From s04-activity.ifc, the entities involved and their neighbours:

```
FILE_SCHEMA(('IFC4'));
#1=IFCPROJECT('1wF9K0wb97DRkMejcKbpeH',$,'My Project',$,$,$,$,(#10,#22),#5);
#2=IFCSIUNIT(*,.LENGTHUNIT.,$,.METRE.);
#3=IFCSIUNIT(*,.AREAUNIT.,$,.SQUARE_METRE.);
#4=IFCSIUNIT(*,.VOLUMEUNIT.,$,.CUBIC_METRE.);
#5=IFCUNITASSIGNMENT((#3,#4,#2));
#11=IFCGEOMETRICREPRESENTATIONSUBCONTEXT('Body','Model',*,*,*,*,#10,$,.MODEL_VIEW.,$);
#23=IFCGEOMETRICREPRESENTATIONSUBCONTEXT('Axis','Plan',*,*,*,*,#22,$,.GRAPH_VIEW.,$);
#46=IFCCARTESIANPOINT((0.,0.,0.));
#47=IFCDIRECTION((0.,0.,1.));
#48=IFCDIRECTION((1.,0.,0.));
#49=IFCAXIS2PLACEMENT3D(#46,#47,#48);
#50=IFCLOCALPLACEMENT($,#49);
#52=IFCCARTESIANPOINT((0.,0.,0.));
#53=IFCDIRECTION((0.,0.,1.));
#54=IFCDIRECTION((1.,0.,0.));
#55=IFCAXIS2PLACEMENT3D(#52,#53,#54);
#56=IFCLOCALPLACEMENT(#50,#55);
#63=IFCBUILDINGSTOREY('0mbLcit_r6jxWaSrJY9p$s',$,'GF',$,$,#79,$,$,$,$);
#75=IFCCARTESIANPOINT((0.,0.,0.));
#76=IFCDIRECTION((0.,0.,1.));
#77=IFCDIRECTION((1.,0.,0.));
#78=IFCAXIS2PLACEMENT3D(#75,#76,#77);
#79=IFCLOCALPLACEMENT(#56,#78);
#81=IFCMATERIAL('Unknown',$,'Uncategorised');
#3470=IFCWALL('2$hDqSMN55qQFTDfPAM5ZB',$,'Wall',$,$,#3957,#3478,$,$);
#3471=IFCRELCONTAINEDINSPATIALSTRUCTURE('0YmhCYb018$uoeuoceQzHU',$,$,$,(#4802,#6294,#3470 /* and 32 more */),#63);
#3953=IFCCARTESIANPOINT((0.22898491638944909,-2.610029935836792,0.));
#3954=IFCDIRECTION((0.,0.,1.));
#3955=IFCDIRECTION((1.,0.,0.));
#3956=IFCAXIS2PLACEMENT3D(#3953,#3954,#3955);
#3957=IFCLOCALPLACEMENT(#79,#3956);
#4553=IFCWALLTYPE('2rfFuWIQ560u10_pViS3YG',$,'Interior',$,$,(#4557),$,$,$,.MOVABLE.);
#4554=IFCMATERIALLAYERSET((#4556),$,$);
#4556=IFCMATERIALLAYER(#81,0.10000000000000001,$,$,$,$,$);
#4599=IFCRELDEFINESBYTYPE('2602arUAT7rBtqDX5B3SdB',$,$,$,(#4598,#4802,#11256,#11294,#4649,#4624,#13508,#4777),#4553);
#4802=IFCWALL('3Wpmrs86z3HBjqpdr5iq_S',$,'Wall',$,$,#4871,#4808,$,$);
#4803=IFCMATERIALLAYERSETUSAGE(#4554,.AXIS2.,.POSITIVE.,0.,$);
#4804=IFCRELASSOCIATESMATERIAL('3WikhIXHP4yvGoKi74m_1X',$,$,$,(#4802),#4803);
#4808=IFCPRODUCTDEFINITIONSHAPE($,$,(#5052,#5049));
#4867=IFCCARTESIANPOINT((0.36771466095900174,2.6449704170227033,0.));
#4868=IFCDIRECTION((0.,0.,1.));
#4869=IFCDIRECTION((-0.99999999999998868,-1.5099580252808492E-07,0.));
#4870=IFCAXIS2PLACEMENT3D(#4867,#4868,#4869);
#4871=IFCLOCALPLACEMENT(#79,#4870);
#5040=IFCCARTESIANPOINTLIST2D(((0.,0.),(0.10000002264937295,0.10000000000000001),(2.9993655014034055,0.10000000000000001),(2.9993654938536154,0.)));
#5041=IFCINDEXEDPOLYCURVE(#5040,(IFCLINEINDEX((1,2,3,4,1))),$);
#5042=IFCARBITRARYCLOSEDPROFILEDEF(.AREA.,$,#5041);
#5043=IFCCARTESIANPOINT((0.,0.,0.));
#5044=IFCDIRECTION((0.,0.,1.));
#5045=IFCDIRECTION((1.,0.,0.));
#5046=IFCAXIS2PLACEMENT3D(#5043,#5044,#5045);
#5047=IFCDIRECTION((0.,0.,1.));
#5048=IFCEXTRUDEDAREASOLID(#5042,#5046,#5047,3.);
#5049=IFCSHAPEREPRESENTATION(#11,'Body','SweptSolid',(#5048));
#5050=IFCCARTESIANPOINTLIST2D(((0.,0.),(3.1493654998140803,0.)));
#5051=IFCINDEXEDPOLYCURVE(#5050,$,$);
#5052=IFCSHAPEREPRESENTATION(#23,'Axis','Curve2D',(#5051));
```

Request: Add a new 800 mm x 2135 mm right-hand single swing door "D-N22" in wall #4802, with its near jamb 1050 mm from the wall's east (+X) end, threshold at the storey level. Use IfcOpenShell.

```python
import numpy as np
import ifcopenshell
import ifcopenshell.api.feature
import ifcopenshell.api.geometry
import ifcopenshell.api.root
import ifcopenshell.api.spatial
import ifcopenshell.geom
import ifcopenshell.util.element
import ifcopenshell.util.placement
import ifcopenshell.util.representation
import ifcopenshell.util.shape
import ifcopenshell.util.unit

model = ifcopenshell.open("s04-activity.ifc")
unit_scale = ifcopenshell.util.unit.calculate_unit_scale(model)
settings = ifcopenshell.geom.settings()


def volume(element):
    """Net volume in cubic metres, openings subtracted."""
    shape = ifcopenshell.geom.create_shape(settings, element)
    return ifcopenshell.util.shape.get_volume(shape.geometry)


wall = model.by_guid("3Wpmrs86z3HBjqpdr5iq_S")
storey = ifcopenshell.util.element.get_container(wall, ifc_class="IfcBuildingStorey")
context = ifcopenshell.util.representation.get_context(model, "Model", "Body", "MODEL_VIEW")
before = volume(wall)

width, height, from_end, sill = 0.8, 2.135, 1.05, 0.0  # metres

# The wall runs along its own X axis, and the end named is its -X end.
wall_shape = ifcopenshell.geom.create_shape(settings, wall)
x, y, z = ifcopenshell.util.shape.get_vertices(wall_shape.geometry).T
start = x.min() + from_end
face, thickness = float(y.min()), float(y.max() - y.min())
wall_matrix = ifcopenshell.util.placement.get_local_placement(wall.ObjectPlacement)
level = ifcopenshell.util.placement.get_local_placement(storey.ObjectPlacement)[2, 3]


def in_wall(x, y):
    """Placement at x, y metres in the wall's axes, at sill height."""
    matrix = wall_matrix.copy()
    matrix[:, 3] = wall_matrix @ np.array([x / unit_scale, y / unit_scale, 0.0, 1.0])
    matrix[2, 3] = level + sill / unit_scale
    return matrix


# Opening: a box that overshoots both wall faces by 50 mm.
opening = ifcopenshell.api.root.create_entity(model, ifc_class="IfcOpeningElement", predefined_type="OPENING")
box = ifcopenshell.api.geometry.add_wall_representation(
    model, context=context, length=width, height=height, thickness=thickness + 0.1
)
ifcopenshell.api.geometry.assign_representation(model, product=opening, representation=box)
ifcopenshell.api.geometry.edit_object_placement(model, product=opening, matrix=in_wall(start, face - 0.05), is_si=False)
ifcopenshell.api.feature.add_feature(model, feature=opening, element=wall)

door = ifcopenshell.api.root.create_entity(model, ifc_class="IfcDoor", name="D-N22", predefined_type="DOOR")
door.OverallWidth, door.OverallHeight = width / unit_scale, height / unit_scale
door.OperationType = "SINGLE_SWING_RIGHT"
body = ifcopenshell.api.geometry.add_door_representation(
    model,
    context=context,
    overall_width=door.OverallWidth,
    overall_height=door.OverallHeight,
    operation_type="SINGLE_SWING_RIGHT",
    lining_properties={"LiningDepth": thickness / unit_scale, "ThresholdDepth": thickness / unit_scale},
)
ifcopenshell.api.geometry.assign_representation(model, product=door, representation=body)
ifcopenshell.api.spatial.assign_container(model, products=[door], relating_structure=storey)
ifcopenshell.api.feature.add_filling(model, opening=opening, element=door)

# The lining spans the wall, so the door starts at the wall face.
ifcopenshell.api.geometry.edit_object_placement(model, product=door, matrix=in_wall(start, face), is_si=False)

after = volume(wall)

print(f"wall volume {before:.3f} -> {after:.3f} m3")

model.write("s04-activity_v2.ifc")
```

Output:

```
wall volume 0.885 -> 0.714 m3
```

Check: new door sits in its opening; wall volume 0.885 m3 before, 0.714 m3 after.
